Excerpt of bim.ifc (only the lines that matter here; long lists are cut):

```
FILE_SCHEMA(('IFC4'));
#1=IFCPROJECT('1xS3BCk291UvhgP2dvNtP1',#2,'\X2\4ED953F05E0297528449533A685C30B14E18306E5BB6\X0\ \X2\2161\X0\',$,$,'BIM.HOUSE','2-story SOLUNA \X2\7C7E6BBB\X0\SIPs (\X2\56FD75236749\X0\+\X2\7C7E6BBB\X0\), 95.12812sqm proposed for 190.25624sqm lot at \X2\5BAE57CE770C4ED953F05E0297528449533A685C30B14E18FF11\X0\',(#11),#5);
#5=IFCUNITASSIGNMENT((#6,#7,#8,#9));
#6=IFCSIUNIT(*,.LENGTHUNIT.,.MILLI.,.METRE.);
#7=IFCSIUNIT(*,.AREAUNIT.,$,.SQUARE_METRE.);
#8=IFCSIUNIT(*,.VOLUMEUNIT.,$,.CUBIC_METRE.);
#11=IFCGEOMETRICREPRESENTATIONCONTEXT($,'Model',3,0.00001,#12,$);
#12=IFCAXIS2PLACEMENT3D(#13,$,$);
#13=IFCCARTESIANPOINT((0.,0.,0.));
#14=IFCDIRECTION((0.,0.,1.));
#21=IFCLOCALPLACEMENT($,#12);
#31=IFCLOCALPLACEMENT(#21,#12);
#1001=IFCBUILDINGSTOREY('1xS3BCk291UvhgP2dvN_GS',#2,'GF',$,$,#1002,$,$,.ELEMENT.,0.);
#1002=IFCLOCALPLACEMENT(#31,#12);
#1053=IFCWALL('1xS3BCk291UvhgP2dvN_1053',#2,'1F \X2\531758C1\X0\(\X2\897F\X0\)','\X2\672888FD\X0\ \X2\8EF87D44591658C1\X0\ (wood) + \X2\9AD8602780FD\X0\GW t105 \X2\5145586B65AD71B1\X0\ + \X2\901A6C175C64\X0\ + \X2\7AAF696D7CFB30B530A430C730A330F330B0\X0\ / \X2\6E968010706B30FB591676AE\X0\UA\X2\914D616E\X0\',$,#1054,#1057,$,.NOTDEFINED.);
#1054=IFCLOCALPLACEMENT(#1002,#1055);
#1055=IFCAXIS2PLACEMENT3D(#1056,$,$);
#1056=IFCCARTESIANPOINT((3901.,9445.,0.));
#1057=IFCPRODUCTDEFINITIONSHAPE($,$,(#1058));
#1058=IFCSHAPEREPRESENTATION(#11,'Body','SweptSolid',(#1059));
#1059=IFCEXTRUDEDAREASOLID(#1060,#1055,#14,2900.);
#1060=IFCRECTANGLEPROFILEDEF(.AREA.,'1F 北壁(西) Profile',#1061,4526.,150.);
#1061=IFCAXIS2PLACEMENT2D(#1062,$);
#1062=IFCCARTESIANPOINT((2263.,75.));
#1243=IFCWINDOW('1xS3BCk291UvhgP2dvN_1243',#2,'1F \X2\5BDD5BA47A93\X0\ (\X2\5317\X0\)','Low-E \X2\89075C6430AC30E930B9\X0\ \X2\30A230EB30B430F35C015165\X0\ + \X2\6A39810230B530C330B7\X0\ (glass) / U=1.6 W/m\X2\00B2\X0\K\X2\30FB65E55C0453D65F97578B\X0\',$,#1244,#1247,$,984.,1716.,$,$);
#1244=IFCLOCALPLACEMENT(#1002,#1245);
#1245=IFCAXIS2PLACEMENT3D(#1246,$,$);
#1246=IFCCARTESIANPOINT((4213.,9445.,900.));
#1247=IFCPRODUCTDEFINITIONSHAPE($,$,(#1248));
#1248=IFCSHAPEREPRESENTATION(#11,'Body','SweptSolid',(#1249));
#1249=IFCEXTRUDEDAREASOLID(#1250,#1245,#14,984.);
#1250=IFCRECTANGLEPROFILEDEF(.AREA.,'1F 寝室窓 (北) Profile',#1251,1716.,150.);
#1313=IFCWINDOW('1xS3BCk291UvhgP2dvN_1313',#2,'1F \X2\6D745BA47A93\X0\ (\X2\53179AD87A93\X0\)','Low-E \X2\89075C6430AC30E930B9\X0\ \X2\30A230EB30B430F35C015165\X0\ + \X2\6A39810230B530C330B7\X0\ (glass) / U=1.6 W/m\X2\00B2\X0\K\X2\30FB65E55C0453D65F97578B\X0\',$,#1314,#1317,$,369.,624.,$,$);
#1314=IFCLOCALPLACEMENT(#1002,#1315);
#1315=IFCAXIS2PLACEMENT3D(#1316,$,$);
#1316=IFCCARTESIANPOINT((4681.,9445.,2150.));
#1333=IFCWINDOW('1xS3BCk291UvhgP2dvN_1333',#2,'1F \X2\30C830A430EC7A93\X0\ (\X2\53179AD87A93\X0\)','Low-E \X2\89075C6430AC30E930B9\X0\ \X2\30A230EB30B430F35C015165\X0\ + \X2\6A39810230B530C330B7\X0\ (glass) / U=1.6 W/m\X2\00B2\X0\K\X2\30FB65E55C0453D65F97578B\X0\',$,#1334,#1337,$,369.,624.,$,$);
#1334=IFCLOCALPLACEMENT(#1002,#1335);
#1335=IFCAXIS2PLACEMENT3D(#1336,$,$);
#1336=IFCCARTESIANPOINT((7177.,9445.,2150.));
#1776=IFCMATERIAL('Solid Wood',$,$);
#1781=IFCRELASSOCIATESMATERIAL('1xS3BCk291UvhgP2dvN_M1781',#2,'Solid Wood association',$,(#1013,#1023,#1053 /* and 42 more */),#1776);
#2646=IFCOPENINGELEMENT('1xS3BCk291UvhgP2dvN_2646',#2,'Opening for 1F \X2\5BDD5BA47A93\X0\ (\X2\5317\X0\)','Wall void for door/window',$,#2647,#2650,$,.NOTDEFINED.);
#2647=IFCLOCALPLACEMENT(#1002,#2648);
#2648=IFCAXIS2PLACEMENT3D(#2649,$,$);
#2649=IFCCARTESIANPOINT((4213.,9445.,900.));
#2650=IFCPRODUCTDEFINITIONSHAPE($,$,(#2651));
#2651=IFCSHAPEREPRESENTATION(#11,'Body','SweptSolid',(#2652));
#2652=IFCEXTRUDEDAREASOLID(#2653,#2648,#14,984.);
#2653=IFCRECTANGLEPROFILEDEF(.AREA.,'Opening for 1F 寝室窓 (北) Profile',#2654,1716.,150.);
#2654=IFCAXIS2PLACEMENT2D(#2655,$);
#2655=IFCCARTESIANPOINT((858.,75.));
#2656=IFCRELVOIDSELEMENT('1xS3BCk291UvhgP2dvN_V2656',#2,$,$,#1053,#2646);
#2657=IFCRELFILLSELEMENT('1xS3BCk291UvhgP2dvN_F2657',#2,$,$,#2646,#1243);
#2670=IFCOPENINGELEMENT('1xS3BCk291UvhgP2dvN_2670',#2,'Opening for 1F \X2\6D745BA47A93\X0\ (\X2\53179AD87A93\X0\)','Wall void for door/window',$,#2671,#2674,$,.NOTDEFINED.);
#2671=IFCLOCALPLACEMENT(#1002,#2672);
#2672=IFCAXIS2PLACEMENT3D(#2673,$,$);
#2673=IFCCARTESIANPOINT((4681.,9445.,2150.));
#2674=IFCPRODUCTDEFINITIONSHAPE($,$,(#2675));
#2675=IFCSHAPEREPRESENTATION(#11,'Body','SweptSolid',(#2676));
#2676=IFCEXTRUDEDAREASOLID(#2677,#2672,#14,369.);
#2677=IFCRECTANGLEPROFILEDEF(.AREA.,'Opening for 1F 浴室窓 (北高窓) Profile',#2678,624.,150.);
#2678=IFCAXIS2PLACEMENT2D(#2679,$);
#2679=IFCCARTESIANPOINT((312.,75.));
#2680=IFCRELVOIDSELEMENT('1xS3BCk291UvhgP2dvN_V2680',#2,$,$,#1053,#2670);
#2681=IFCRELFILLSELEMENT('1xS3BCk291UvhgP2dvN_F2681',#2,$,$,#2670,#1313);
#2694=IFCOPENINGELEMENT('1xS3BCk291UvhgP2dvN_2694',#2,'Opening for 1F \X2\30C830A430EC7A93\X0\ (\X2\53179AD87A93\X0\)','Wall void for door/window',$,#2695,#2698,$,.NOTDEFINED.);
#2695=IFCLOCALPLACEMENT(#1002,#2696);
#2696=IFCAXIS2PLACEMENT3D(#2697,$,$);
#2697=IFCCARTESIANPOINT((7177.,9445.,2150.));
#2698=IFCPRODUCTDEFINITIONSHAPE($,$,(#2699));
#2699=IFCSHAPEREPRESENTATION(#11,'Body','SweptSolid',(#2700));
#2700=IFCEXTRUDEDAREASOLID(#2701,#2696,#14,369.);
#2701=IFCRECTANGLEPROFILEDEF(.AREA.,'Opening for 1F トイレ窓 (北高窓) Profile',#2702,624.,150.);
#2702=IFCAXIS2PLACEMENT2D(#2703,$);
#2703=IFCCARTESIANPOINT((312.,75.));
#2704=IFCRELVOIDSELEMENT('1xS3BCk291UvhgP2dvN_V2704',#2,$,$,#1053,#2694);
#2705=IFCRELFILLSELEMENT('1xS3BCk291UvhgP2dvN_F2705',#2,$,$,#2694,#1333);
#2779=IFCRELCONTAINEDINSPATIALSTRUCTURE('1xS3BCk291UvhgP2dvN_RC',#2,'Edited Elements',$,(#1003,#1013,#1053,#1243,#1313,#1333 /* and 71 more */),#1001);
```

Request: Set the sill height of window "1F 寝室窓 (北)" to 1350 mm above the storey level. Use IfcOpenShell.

```python
import numpy as np
import ifcopenshell
import ifcopenshell.api.geometry
import ifcopenshell.geom
import ifcopenshell.util.element
import ifcopenshell.util.placement
import ifcopenshell.util.shape
import ifcopenshell.util.unit

model = ifcopenshell.open("bim.ifc")
unit_scale = ifcopenshell.util.unit.calculate_unit_scale(model)

window = model.by_id(1243)
opening = window.FillsVoids[0].RelatingOpeningElement
storey = ifcopenshell.util.element.get_container(window, ifc_class="IfcBuildingStorey")
level = ifcopenshell.util.placement.get_local_placement(storey.ObjectPlacement)[2, 3]

# The opening's origin need not be at the sill, so measure its lowest point.
shape = ifcopenshell.geom.create_shape(ifcopenshell.geom.settings(), opening)
bottom = ifcopenshell.util.shape.get_shape_bottom_elevation(shape, shape.geometry) / unit_scale
dz = level + 1.35 / unit_scale - bottom

shift = np.array([0.0, 0.0, dz])
# The window is not placed relative to its opening, so move both.
for product in (opening, window):
    matrix = ifcopenshell.util.placement.get_local_placement(product.ObjectPlacement)
    matrix[:3, 3] += shift
    ifcopenshell.api.geometry.edit_object_placement(model, product=product, matrix=matrix, is_si=False)

print(f"moved by {dz * unit_scale:+.3f} m")

model.write("bim_rev.ifc")
```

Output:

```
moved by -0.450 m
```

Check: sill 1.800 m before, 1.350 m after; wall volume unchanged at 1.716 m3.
